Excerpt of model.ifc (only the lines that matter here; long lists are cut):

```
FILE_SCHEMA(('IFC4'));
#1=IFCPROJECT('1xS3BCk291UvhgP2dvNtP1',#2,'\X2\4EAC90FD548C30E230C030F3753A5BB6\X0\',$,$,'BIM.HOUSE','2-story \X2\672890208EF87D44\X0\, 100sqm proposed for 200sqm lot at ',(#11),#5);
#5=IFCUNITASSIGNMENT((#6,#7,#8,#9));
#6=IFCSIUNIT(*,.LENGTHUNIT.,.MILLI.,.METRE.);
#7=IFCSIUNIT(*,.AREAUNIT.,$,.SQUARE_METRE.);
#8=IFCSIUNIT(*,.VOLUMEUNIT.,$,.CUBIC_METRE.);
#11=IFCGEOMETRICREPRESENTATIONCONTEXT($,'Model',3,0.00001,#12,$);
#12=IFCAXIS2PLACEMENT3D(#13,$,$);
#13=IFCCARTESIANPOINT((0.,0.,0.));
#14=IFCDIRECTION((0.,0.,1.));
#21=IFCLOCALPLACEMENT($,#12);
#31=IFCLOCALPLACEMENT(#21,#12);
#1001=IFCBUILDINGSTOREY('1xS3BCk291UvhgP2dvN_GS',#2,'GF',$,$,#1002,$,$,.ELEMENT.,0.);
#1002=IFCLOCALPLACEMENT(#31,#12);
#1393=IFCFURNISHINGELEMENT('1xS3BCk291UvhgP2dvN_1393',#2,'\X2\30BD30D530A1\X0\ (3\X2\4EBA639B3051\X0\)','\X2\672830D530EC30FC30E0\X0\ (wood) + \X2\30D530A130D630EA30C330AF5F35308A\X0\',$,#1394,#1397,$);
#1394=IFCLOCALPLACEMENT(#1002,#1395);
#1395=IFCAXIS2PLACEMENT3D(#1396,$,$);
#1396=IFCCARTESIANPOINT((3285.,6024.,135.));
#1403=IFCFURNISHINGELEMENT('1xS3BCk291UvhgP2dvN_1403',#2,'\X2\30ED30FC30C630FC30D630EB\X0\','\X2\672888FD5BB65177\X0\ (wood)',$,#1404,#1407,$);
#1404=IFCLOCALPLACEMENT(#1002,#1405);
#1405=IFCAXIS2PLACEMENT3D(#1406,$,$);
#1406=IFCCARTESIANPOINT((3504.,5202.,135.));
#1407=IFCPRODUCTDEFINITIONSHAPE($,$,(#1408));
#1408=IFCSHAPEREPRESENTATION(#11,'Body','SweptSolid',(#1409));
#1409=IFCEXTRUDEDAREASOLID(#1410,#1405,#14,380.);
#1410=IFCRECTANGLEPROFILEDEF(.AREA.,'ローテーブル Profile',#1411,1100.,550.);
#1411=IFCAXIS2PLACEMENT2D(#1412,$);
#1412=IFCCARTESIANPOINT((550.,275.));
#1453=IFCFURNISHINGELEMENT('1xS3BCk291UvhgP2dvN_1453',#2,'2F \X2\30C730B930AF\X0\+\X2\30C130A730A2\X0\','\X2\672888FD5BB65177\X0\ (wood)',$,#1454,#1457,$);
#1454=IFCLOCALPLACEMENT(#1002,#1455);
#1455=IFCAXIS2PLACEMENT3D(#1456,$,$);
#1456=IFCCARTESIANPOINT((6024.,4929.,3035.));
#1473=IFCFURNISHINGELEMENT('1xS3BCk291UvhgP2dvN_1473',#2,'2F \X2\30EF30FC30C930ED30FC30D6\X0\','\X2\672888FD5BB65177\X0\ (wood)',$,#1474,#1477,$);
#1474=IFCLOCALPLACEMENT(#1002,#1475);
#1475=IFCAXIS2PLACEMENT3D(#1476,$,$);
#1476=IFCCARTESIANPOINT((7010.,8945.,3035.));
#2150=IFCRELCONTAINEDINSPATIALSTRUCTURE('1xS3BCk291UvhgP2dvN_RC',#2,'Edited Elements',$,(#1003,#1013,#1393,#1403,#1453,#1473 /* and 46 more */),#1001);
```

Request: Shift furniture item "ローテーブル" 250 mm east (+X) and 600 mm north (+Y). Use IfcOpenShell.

```python
import ifcopenshell
import ifcopenshell.api.geometry
import ifcopenshell.util.placement

model = ifcopenshell.open("model.ifc")

item = model.by_guid("1xS3BCk291UvhgP2dvN_1403")
matrix = ifcopenshell.util.placement.get_local_placement(item.ObjectPlacement)
matrix[0, 3] += 250.0
matrix[1, 3] += 600.0
ifcopenshell.api.geometry.edit_object_placement(model, product=item, matrix=matrix, is_si=False)

print(ifcopenshell.util.placement.get_local_placement(item.ObjectPlacement).round(3) + 0.0)

model.write("model_v2.ifc")
```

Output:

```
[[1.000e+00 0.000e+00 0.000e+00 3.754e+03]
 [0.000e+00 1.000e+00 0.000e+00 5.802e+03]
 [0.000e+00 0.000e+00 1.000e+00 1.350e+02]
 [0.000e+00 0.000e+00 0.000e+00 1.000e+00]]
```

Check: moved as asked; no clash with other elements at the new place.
